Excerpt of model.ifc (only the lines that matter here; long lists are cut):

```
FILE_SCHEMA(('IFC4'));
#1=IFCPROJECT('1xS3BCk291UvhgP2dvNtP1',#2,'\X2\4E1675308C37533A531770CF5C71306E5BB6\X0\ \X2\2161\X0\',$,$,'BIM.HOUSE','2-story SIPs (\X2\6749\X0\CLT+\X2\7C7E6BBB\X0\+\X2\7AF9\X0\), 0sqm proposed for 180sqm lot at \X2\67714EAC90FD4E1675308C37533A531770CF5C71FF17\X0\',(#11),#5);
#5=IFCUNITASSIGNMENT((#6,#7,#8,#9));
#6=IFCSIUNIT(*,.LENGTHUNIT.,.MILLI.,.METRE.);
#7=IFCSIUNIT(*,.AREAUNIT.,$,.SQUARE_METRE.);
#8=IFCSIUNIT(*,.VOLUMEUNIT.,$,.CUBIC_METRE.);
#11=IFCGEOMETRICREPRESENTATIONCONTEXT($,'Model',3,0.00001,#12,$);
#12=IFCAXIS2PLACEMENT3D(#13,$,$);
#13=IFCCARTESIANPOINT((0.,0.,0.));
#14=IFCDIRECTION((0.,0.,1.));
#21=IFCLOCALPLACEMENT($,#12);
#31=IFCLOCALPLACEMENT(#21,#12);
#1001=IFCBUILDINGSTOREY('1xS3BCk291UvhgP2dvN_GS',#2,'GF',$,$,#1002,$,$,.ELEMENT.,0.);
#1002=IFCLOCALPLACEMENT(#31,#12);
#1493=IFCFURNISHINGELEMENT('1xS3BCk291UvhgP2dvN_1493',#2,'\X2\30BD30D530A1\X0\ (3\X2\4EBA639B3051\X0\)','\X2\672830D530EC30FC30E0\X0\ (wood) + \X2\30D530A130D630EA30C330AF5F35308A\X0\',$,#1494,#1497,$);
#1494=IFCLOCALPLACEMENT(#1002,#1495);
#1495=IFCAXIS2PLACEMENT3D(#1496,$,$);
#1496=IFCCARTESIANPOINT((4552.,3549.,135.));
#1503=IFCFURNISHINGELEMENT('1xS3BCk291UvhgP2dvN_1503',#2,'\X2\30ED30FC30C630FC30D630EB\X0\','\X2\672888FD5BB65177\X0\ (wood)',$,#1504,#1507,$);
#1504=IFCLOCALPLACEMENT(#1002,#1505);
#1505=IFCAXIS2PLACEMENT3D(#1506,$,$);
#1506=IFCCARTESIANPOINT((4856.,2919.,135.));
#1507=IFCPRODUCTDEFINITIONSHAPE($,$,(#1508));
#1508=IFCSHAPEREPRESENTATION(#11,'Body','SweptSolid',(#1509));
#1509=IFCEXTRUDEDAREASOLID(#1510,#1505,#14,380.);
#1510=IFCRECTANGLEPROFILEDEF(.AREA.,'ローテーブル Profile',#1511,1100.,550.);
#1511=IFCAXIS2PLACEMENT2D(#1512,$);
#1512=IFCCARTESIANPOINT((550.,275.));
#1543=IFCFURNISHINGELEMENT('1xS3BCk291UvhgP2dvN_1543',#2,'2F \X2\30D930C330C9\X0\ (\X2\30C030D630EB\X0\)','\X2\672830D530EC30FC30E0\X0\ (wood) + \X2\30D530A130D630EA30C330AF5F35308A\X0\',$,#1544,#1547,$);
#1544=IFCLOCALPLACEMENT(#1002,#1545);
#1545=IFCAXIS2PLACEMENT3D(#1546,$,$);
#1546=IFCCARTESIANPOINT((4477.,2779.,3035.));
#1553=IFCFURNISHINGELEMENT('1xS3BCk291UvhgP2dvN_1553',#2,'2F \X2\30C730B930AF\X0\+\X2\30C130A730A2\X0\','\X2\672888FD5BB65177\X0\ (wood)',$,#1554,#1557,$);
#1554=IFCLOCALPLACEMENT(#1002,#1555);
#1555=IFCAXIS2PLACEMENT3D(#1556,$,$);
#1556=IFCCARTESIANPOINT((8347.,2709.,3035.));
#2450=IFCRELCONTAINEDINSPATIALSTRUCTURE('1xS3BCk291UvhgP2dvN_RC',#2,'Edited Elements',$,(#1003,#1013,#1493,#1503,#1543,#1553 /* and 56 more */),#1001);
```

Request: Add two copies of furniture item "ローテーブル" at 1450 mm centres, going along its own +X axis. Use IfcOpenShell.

```python
import ifcopenshell
import ifcopenshell.api.geometry
import ifcopenshell.api.root
import ifcopenshell.util.element
import ifcopenshell.util.placement
import ifcopenshell.util.unit

model = ifcopenshell.open("model.ifc")
unit_scale = ifcopenshell.util.unit.calculate_unit_scale(model)


def reuse_history(source, copy):
    """copy_class also copies each property set's owner history, people and application; keep the originals."""
    for rel in copy.IsDefinedBy:
        if rel.is_a("IfcRelDefinesByProperties") and (history := rel.RelatingPropertyDefinition.OwnerHistory):
            rel.RelatingPropertyDefinition.OwnerHistory = source.OwnerHistory
            ifcopenshell.util.element.remove_deep2(model, history)


source = model.by_guid("1xS3BCk291UvhgP2dvN_1503")
base = ifcopenshell.util.placement.get_local_placement(source.ObjectPlacement)
step = base[:3, 0] * 1.45 / unit_scale

for i in range(1, 3):
    copy = ifcopenshell.api.root.copy_class(model, product=source)
    copy.Representation = ifcopenshell.util.element.copy_deep(
        model, source.Representation, exclude=["IfcGeometricRepresentationContext", "IfcRepresentationMap"]
    )
    reuse_history(source, copy)
    matrix = base.copy()
    matrix[:3, 3] += i * step
    print("added at", matrix[:3, 3].round(3) + 0.0)
    ifcopenshell.api.geometry.edit_object_placement(model, product=copy, matrix=matrix, is_si=False)

model.write("model_edited.ifc")
```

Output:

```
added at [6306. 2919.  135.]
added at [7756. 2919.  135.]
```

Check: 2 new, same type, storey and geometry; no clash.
